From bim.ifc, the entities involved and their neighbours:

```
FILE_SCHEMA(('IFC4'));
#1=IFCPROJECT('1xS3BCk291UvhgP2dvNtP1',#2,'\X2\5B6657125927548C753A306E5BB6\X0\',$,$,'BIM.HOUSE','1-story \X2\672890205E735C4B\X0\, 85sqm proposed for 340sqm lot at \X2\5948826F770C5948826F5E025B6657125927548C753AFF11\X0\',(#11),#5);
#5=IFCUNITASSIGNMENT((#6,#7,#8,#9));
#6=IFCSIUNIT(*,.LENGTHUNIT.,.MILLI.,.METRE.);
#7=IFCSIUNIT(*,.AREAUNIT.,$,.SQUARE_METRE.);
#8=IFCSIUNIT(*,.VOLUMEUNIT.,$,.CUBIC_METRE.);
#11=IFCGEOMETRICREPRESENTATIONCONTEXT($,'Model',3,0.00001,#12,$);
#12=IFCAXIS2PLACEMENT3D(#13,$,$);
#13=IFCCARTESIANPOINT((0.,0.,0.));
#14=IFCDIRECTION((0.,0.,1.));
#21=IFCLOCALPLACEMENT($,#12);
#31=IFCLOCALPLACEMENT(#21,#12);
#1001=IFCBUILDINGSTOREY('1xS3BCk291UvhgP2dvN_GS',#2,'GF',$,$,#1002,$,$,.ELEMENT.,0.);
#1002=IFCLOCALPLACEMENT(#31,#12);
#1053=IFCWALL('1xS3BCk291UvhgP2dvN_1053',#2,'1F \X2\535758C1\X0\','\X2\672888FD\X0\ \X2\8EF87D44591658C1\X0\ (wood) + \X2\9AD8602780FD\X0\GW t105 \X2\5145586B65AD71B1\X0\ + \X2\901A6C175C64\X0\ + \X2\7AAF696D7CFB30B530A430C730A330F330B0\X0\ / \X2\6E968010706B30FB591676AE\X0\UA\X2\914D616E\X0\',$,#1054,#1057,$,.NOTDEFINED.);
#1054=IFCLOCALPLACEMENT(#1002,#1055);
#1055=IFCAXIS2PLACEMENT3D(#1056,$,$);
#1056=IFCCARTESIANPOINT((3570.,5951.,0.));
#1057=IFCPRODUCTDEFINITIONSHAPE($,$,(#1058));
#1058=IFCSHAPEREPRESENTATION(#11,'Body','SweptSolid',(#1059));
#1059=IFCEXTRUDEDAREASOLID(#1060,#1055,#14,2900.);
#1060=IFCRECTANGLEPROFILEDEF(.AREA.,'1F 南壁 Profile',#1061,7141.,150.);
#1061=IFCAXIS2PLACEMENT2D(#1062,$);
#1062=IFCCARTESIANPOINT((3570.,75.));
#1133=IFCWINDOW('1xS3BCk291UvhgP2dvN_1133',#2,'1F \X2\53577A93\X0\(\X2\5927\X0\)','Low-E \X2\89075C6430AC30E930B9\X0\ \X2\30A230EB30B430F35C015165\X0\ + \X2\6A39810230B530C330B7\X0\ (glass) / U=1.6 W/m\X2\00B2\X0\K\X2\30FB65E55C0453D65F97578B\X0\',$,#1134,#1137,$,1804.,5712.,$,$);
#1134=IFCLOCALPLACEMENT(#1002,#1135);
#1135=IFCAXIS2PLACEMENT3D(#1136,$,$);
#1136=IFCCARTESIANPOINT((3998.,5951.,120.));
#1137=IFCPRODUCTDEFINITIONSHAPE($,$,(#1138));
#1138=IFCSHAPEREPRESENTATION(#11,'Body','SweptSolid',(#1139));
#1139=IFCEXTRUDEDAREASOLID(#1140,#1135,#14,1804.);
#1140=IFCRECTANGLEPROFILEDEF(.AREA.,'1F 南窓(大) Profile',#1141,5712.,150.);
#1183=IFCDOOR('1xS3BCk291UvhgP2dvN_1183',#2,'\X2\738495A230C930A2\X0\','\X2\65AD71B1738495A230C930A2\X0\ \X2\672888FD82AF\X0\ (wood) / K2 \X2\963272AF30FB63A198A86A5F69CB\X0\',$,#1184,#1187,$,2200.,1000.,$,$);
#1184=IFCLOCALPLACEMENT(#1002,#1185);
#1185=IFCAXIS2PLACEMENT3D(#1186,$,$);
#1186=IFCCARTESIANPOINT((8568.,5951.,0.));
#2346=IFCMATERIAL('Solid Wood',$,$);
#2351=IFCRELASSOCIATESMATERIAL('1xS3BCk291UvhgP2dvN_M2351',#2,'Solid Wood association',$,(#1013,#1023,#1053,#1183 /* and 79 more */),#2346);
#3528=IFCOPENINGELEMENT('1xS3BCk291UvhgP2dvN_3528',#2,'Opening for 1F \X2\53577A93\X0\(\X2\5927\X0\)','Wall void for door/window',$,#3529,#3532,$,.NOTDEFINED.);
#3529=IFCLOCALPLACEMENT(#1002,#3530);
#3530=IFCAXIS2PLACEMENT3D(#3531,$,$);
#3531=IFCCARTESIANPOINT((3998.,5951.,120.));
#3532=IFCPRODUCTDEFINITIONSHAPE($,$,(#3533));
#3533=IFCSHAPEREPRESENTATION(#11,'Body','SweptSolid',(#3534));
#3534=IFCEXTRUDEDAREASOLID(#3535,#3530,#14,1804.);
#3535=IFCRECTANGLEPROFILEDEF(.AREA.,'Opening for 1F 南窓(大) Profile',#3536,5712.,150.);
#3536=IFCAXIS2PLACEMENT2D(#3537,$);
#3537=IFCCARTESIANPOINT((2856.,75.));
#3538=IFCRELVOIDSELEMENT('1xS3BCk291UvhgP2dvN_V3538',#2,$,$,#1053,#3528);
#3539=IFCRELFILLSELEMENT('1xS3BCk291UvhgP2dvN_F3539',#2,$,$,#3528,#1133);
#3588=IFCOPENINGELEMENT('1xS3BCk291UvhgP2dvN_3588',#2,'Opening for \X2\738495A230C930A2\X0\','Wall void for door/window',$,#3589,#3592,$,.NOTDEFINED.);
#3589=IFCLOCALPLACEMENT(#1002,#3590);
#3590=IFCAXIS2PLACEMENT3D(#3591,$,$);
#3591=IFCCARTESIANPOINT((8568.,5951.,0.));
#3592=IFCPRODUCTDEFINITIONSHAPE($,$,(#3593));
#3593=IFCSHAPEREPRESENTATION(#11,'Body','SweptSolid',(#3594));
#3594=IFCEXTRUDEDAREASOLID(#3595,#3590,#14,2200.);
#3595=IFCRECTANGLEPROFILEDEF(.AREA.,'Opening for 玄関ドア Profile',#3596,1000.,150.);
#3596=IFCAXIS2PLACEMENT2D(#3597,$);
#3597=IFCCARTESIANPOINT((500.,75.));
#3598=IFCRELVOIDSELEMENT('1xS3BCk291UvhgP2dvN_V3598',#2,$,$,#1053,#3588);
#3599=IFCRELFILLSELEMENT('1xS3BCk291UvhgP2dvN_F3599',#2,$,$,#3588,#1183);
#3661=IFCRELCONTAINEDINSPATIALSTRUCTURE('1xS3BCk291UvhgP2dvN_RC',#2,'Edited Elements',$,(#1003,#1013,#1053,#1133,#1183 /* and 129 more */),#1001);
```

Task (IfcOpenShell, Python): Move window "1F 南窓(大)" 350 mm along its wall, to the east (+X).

```python
import ifcopenshell
import ifcopenshell.api.geometry
import ifcopenshell.util.placement

model = ifcopenshell.open("bim.ifc")

window = model.by_guid("1xS3BCk291UvhgP2dvN_1133")
opening = window.FillsVoids[0].RelatingOpeningElement
wall = opening.VoidsElements[0].RelatingBuildingElement

wall_matrix = ifcopenshell.util.placement.get_local_placement(wall.ObjectPlacement)
shift = wall_matrix[:3, 0] * 350.0
before = ifcopenshell.util.placement.get_local_placement(window.ObjectPlacement)[:3, 3].copy()

# The window is not placed relative to its opening, so move both.
for product in (opening, window):
    matrix = ifcopenshell.util.placement.get_local_placement(product.ObjectPlacement)
    matrix[:3, 3] += shift
    ifcopenshell.api.geometry.edit_object_placement(model, product=product, matrix=matrix, is_si=False)

after = ifcopenshell.util.placement.get_local_placement(window.ObjectPlacement)[:3, 3]
print("window moved by", (after - before).round(3) + 0.0)

model.write("bim_rev.ifc")
```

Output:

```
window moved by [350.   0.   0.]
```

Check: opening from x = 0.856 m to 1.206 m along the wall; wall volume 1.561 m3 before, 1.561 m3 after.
